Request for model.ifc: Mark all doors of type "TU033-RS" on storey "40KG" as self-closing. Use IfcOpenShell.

First a look at what the model holds.

```python
import ifcopenshell
import ifcopenshell.util.element

model = ifcopenshell.open("model.ifc")
print(model.schema)
storey = next(s for s in model.by_type("IfcBuildingStorey") if s.Name == "40KG")
doors = [e for e in ifcopenshell.util.element.get_decomposition(storey) if e.is_a("IfcDoor")]
seen = {}
for e in doors:
    element_type = ifcopenshell.util.element.get_type(e)
    key = (element_type.Name if element_type != e and element_type else None, ifcopenshell.util.element.get_pset(e, "Pset_DoorCommon", "SelfClosing"))
    seen[key] = seen.get(key, 0) + 1
for (name, value), count in sorted(seen.items(), key=str):
    print(count, "x", name, "|", value)
```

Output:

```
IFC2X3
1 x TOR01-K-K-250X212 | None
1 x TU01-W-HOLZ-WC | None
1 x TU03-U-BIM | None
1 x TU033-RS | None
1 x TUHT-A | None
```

```python
import ifcopenshell
import ifcopenshell.api.pset
import ifcopenshell.util.element

model = ifcopenshell.open("model.ifc")

storey = next(s for s in model.by_type("IfcBuildingStorey") if s.Name == "40KG")
doors = [e for e in ifcopenshell.util.element.get_decomposition(storey) if e.is_a("IfcDoor")]

count = 0
for e in doors:
    element_type = ifcopenshell.util.element.get_type(e)
    if element_type in (None, e) or element_type.Name != "TU033-RS":
        continue
    # add_pset returns the element's existing set when there is one.
    pset = ifcopenshell.api.pset.add_pset(model, product=e, name="Pset_DoorCommon")
    ifcopenshell.api.pset.edit_pset(model, pset=pset, properties={"SelfClosing": True})
    count += 1

print(count, "doors updated")

model.write("model_updated.ifc")
```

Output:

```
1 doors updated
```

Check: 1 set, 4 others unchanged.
